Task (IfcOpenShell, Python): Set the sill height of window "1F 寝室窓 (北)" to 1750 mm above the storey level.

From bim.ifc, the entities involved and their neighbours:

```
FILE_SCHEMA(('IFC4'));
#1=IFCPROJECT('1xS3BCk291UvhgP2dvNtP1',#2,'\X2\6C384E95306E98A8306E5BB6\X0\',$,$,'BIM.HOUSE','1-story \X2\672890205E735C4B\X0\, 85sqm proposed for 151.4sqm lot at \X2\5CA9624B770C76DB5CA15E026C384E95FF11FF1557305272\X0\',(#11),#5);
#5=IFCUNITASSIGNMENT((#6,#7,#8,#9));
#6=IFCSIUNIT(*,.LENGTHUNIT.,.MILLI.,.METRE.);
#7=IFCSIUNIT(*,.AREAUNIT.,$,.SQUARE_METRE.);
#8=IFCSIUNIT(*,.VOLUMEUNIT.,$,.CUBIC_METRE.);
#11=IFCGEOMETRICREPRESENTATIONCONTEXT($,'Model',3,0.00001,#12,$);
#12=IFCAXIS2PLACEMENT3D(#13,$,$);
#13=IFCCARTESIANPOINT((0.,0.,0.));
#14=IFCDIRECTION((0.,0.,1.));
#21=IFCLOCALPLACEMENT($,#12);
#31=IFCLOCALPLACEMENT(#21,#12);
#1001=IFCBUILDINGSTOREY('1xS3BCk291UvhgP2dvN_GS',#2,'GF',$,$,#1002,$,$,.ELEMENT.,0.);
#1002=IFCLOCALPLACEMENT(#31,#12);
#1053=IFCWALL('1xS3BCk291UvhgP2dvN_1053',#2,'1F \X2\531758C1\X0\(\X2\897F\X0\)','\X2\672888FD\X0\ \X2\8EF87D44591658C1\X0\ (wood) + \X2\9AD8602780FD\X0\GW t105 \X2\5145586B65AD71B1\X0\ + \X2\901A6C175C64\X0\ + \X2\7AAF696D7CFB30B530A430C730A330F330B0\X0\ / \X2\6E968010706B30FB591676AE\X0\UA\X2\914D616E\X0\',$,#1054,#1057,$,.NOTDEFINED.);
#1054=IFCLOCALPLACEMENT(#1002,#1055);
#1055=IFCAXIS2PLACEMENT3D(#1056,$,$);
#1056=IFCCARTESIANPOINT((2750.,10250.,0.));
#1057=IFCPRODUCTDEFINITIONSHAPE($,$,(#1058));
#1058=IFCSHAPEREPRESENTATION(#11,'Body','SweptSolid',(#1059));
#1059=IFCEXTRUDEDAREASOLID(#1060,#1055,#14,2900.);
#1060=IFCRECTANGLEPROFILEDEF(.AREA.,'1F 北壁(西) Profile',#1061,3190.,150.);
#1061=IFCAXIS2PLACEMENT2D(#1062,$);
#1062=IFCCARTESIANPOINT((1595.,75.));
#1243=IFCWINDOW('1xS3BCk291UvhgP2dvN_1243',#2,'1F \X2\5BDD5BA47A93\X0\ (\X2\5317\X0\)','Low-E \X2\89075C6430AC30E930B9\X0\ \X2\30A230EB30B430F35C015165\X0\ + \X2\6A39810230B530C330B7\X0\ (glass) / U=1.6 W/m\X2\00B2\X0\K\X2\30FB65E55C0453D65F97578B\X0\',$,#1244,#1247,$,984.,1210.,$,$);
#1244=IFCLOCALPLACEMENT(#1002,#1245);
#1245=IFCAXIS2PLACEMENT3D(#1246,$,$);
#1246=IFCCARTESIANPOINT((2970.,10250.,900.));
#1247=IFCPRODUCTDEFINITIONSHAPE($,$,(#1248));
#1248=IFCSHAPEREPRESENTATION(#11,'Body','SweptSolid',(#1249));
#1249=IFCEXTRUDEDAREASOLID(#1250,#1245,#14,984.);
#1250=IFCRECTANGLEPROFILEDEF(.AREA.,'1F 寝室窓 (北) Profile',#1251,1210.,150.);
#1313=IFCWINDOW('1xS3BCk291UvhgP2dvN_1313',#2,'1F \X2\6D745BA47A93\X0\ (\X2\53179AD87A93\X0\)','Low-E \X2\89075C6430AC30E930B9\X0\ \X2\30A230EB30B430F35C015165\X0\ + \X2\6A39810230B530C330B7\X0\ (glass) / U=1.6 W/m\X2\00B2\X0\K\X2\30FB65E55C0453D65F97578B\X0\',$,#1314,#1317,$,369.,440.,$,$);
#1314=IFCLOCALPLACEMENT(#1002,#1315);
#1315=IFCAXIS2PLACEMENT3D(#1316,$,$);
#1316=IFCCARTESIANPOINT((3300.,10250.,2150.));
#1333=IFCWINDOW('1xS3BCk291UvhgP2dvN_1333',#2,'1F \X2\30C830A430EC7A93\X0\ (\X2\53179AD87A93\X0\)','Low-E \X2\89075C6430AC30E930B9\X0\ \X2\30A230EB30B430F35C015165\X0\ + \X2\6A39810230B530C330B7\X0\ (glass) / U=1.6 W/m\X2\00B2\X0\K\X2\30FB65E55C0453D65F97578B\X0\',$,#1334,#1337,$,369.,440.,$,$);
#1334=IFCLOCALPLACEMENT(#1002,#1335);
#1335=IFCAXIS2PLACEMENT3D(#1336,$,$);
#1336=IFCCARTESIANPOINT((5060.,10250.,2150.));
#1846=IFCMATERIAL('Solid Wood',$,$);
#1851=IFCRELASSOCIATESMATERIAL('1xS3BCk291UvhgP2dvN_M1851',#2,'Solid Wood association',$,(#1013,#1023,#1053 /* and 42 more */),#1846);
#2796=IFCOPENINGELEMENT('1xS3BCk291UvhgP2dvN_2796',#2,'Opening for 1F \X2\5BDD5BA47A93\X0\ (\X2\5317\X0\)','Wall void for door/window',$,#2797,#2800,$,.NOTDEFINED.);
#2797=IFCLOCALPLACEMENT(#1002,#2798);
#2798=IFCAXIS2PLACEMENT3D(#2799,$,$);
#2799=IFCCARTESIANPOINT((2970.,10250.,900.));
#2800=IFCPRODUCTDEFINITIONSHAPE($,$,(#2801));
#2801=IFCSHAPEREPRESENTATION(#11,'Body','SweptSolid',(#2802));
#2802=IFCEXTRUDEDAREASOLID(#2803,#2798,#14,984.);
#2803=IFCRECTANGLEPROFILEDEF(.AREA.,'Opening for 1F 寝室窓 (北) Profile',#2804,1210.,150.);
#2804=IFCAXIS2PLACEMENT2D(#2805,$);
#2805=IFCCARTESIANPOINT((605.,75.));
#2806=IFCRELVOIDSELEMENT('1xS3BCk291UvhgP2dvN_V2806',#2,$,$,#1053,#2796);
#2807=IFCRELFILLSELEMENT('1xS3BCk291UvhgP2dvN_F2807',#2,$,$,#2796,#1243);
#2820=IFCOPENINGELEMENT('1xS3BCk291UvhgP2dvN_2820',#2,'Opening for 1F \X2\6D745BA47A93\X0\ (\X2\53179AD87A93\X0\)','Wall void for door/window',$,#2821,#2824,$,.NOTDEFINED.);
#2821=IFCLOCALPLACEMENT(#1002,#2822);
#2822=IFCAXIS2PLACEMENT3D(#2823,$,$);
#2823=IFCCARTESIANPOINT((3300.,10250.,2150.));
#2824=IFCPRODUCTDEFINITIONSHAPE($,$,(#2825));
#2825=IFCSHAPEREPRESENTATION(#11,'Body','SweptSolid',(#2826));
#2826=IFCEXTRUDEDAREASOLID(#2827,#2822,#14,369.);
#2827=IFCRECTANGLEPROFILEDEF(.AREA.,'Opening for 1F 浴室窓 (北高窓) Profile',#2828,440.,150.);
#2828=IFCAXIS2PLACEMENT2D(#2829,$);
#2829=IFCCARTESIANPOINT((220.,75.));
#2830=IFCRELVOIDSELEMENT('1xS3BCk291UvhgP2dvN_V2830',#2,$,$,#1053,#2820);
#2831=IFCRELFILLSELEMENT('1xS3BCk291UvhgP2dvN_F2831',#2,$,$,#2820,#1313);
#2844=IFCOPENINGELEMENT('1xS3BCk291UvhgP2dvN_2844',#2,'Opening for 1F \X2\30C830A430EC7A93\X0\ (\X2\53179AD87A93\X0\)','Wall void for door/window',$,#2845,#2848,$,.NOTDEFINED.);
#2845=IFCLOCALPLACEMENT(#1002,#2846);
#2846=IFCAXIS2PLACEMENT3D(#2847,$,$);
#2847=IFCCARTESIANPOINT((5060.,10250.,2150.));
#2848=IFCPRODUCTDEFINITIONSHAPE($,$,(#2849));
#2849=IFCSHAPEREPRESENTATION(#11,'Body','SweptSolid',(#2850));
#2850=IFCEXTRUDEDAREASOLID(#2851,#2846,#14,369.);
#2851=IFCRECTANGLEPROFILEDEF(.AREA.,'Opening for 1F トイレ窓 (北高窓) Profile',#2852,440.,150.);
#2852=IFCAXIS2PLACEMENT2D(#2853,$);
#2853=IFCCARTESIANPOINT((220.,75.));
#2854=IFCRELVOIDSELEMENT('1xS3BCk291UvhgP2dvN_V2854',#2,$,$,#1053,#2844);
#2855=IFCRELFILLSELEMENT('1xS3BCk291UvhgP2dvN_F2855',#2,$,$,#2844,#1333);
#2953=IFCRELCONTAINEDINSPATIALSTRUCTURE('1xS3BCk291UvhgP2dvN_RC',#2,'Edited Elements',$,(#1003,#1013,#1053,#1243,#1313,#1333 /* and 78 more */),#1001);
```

```python
import numpy as np
import ifcopenshell
import ifcopenshell.api.geometry
import ifcopenshell.geom
import ifcopenshell.util.element
import ifcopenshell.util.placement
import ifcopenshell.util.shape
import ifcopenshell.util.unit

model = ifcopenshell.open("bim.ifc")
unit_scale = ifcopenshell.util.unit.calculate_unit_scale(model)

window = model.by_guid("1xS3BCk291UvhgP2dvN_1243")
opening = window.FillsVoids[0].RelatingOpeningElement
storey = ifcopenshell.util.element.get_container(window, ifc_class="IfcBuildingStorey")
level = ifcopenshell.util.placement.get_local_placement(storey.ObjectPlacement)[2, 3]

# The opening's origin need not be at the sill, so measure its lowest point.
shape = ifcopenshell.geom.create_shape(ifcopenshell.geom.settings(), opening)
bottom = ifcopenshell.util.shape.get_shape_bottom_elevation(shape, shape.geometry) / unit_scale
dz = level + 1.75 / unit_scale - bottom

shift = np.array([0.0, 0.0, dz])
# The window is not placed relative to its opening, so move both.
for product in (opening, window):
    matrix = ifcopenshell.util.placement.get_local_placement(product.ObjectPlacement)
    matrix[:3, 3] += shift
    ifcopenshell.api.geometry.edit_object_placement(model, product=product, matrix=matrix, is_si=False)

print(f"moved by {dz * unit_scale:+.3f} m")

model.write("bim-out.ifc")
```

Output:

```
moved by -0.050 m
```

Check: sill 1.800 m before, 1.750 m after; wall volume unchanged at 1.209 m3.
